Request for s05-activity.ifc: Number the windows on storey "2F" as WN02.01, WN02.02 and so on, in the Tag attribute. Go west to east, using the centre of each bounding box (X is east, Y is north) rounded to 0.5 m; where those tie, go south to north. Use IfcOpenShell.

First a look at what the model holds.

```python
import ifcopenshell
import ifcopenshell.util.element
import ifcopenshell.util.placement

model = ifcopenshell.open("s05-activity.ifc")
print(model.schema)
storey = next(s for s in model.by_type("IfcBuildingStorey") if s.Name == "2F")
windows = [e for e in ifcopenshell.util.element.get_decomposition(storey) if e.is_a("IfcWindow")]
for e in sorted(windows, key=lambda e: e.id()):
    origin = ifcopenshell.util.placement.get_local_placement(e.ObjectPlacement)[:3, 3]
    print(e.id(), e.Tag, e.Name, origin.round(2) + 0.0, sep=" | ")
```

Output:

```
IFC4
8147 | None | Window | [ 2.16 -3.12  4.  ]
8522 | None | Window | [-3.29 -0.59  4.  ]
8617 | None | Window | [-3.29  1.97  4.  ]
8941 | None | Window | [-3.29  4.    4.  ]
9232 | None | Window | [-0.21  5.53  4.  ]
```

```python
import ifcopenshell
import ifcopenshell.geom
import ifcopenshell.util.element
import ifcopenshell.util.shape

model = ifcopenshell.open("s05-activity.ifc")
settings = ifcopenshell.geom.settings()
settings.set("use-world-coords", True)


def centre(element):
    shape = ifcopenshell.geom.create_shape(settings, element)
    return ifcopenshell.util.shape.get_bbox_centroid(shape.geometry)


storey = next(s for s in model.by_type("IfcBuildingStorey") if s.Name == "2F")
windows = [e for e in ifcopenshell.util.element.get_decomposition(storey) if e.is_a("IfcWindow")]

# Insertion points can sit at a corner or the storey origin, so sort by the geometry (in metres).
centres = {e: centre(e) for e in windows}
windows.sort(key=lambda e: (round(centres[e][0] / 0.5), centres[e][1]))

for i, e in enumerate(windows, start=1):
    number = f"WN02.{i:02d}"
    e.Tag = number
    print(e.id(), number)

model.write("s05-activity_v2.ifc")
```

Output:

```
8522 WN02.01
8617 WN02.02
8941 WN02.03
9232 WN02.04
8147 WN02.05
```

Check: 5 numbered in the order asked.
